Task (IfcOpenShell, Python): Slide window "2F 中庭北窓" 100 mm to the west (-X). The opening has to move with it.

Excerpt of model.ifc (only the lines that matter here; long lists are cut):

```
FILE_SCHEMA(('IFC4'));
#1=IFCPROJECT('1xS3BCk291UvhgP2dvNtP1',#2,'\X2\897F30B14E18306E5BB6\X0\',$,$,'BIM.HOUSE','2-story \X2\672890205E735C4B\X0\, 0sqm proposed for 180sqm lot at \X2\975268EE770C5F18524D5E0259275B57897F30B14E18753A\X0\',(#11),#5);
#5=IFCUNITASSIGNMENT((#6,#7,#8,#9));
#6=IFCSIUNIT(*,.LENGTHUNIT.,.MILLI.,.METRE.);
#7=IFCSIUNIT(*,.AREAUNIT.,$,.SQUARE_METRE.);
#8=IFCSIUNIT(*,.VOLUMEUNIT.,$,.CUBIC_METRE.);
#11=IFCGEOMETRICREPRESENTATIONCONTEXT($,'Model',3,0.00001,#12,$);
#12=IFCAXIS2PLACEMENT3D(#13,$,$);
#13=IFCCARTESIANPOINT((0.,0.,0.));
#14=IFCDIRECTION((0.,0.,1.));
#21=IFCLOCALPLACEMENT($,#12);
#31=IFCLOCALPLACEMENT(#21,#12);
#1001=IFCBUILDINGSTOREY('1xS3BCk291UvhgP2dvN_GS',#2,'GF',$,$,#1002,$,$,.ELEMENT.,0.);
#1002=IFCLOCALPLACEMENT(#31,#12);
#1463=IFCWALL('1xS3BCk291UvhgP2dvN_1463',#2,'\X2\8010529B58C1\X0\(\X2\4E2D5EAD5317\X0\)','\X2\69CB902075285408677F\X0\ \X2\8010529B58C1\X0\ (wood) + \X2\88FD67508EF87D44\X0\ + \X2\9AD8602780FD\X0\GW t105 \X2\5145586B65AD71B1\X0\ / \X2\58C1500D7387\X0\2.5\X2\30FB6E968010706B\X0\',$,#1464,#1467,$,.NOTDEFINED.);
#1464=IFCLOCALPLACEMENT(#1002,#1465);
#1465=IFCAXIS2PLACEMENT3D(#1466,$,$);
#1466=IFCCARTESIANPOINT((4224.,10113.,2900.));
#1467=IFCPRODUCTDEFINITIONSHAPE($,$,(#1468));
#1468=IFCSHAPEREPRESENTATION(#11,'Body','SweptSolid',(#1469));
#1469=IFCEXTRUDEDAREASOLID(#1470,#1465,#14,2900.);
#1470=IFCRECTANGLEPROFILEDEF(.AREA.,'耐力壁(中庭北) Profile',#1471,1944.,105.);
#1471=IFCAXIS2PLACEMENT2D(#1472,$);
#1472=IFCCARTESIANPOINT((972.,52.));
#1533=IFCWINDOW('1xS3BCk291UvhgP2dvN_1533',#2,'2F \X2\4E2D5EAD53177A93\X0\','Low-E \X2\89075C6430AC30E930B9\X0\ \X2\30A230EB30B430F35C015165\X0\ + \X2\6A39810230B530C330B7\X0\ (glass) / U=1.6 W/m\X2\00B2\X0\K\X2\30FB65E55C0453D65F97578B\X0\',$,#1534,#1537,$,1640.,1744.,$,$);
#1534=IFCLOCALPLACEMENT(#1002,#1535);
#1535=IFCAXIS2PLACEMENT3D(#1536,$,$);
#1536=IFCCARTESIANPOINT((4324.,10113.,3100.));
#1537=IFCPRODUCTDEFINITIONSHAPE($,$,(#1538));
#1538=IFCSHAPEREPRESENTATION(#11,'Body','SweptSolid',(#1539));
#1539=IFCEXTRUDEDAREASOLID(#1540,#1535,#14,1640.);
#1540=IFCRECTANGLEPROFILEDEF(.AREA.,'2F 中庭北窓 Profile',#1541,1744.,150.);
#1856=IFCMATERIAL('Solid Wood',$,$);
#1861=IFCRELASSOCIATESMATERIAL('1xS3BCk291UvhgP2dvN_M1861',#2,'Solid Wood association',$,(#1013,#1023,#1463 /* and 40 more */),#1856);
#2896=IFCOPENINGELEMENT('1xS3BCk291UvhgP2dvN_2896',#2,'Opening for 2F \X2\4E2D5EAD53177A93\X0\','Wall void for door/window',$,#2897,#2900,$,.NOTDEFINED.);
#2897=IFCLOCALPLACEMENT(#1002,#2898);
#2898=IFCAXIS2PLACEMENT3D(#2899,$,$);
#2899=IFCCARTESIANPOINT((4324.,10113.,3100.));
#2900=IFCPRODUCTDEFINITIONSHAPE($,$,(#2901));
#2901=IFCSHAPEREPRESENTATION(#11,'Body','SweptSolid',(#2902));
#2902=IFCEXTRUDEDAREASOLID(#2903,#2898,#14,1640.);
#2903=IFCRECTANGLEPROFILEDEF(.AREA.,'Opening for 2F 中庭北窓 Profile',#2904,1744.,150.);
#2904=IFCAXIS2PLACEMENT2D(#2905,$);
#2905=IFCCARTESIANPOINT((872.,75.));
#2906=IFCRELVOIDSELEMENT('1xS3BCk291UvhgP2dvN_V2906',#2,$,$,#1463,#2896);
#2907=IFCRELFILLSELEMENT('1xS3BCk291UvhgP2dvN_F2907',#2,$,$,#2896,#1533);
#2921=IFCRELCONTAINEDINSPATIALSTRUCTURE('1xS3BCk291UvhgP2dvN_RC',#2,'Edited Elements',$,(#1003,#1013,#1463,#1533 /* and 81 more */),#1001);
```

```python
import ifcopenshell
import ifcopenshell.api.geometry
import ifcopenshell.util.placement
import ifcopenshell.util.unit

model = ifcopenshell.open("model.ifc")
unit_scale = ifcopenshell.util.unit.calculate_unit_scale(model)

window = model.by_guid("1xS3BCk291UvhgP2dvN_1533")
opening = window.FillsVoids[0].RelatingOpeningElement
wall = opening.VoidsElements[0].RelatingBuildingElement

wall_matrix = ifcopenshell.util.placement.get_local_placement(wall.ObjectPlacement)
shift = wall_matrix[:3, 0] * -0.1 / unit_scale
before = ifcopenshell.util.placement.get_local_placement(window.ObjectPlacement)[:3, 3].copy()

# The window is not placed relative to its opening, so move both.
for product in (opening, window):
    matrix = ifcopenshell.util.placement.get_local_placement(product.ObjectPlacement)
    matrix[:3, 3] += shift
    ifcopenshell.api.geometry.edit_object_placement(model, product=product, matrix=matrix, is_si=False)

after = ifcopenshell.util.placement.get_local_placement(window.ObjectPlacement)[:3, 3]
print("window moved by", (after - before).round(3) + 0.0)

model.write("model-out.ifc")
```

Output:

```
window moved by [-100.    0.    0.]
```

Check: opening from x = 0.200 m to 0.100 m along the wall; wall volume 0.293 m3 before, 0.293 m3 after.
